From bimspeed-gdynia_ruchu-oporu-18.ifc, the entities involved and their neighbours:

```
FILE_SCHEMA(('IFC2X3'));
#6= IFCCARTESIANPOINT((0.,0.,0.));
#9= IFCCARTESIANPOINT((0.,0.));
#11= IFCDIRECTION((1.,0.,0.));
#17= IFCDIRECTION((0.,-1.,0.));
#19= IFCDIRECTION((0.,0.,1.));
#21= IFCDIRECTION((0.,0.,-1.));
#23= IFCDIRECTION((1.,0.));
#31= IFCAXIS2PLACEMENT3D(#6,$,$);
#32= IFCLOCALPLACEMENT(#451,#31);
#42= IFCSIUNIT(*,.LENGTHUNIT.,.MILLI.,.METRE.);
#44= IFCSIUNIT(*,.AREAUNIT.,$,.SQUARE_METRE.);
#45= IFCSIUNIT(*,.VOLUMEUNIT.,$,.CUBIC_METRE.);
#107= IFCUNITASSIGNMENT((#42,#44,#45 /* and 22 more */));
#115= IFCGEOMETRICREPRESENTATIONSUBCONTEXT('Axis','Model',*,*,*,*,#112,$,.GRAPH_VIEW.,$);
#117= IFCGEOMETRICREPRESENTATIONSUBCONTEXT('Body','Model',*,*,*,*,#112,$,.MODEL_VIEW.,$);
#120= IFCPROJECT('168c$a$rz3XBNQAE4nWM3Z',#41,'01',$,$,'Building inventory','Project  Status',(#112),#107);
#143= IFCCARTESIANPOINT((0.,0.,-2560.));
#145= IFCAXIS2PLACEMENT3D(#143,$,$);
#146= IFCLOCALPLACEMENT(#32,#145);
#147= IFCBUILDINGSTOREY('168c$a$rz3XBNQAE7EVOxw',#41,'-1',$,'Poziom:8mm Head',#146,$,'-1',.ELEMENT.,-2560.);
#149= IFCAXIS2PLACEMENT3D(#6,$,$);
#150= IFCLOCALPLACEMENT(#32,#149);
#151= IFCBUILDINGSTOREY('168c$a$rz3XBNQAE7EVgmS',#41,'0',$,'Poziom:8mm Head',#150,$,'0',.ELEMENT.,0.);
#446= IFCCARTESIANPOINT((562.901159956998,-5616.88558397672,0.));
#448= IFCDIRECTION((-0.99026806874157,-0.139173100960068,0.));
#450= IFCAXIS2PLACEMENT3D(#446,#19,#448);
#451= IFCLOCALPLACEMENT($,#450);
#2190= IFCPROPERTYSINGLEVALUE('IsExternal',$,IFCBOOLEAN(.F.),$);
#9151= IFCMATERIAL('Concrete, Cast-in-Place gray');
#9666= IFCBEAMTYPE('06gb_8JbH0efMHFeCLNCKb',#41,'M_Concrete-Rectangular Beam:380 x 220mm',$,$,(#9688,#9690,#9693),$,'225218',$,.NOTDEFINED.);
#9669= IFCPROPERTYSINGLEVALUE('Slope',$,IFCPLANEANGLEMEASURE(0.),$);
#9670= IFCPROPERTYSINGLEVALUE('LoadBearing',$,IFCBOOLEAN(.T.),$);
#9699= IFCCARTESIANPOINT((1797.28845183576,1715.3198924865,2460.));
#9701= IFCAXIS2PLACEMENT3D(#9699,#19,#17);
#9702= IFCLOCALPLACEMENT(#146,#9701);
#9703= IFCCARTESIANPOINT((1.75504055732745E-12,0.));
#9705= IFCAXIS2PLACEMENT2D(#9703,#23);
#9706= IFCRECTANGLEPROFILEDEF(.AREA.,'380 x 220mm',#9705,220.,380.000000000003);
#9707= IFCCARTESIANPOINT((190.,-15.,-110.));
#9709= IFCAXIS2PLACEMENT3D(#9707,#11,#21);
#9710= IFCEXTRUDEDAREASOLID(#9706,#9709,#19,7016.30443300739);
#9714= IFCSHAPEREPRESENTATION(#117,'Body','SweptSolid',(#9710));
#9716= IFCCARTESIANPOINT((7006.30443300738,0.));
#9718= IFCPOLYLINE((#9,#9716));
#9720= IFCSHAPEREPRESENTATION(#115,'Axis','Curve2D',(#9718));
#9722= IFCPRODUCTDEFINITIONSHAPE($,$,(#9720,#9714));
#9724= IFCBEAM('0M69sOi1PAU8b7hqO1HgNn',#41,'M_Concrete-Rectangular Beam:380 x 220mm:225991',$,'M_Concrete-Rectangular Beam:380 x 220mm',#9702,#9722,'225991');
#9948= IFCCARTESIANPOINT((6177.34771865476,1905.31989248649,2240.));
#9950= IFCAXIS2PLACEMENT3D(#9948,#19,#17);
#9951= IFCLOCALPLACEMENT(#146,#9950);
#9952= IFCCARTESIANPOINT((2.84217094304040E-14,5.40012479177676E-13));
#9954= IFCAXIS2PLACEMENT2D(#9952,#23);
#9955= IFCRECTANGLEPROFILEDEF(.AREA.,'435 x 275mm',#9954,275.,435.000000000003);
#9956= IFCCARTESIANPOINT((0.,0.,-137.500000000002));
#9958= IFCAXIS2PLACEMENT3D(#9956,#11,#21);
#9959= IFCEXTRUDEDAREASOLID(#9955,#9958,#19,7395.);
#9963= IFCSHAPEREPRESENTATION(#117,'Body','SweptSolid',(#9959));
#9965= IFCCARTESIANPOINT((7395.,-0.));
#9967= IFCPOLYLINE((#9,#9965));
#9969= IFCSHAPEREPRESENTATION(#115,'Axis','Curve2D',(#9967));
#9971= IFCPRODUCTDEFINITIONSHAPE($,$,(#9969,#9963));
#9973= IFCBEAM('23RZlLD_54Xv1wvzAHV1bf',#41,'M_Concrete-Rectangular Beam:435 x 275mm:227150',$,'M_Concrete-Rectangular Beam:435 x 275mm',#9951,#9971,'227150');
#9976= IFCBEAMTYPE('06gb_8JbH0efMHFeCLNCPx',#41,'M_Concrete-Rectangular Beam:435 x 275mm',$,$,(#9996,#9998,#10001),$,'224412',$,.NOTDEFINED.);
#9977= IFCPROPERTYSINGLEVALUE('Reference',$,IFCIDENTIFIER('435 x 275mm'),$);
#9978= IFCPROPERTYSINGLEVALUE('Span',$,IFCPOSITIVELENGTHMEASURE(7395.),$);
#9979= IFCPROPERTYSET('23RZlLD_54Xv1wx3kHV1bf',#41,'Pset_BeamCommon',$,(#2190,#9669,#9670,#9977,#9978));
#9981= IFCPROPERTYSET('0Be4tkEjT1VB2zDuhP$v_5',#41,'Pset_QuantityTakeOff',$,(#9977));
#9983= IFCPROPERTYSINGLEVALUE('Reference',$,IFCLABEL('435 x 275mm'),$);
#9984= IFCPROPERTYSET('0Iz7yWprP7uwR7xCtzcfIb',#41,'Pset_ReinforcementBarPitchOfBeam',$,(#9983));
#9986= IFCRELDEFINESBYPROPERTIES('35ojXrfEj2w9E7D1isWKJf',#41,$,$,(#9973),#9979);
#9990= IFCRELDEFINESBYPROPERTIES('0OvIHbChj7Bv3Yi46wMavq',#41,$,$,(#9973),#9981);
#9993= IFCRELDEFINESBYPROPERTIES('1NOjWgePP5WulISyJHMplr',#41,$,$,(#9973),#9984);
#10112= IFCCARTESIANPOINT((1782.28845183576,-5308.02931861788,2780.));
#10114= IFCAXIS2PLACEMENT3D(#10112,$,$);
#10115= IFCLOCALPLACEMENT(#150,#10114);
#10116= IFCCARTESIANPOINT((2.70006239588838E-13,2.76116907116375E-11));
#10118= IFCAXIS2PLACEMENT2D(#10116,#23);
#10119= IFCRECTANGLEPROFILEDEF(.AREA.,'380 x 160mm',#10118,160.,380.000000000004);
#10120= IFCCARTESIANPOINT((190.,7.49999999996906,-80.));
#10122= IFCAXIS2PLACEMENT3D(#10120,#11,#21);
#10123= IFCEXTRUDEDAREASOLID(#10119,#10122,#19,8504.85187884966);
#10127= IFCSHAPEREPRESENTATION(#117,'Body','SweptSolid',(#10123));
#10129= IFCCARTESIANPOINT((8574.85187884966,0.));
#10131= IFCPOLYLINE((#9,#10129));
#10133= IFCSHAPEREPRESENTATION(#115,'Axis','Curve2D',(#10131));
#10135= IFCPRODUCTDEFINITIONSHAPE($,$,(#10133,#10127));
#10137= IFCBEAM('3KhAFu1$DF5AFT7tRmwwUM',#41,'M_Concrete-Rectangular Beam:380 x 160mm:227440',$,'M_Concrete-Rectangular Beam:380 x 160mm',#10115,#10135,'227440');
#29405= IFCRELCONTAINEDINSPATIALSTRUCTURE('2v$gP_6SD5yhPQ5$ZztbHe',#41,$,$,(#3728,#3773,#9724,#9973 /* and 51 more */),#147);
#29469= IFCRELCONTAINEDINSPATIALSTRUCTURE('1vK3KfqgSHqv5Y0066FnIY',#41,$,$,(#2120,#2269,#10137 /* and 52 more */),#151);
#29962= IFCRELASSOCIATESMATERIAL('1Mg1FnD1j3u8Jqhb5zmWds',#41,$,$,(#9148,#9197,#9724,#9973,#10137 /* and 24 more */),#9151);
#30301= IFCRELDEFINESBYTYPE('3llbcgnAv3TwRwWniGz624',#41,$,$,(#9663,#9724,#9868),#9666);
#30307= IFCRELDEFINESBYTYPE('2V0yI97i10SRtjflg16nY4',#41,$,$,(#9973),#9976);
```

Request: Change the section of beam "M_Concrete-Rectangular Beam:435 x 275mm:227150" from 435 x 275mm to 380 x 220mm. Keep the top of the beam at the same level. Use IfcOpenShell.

```python
import ifcopenshell
import ifcopenshell.api.pset
import ifcopenshell.api.type
import ifcopenshell.util.element
import ifcopenshell.util.representation

model = ifcopenshell.open("bimspeed-gdynia_ruchu-oporu-18.ifc")

member = model.by_guid("23RZlLD_54Xv1wvzAHV1bf")
source = next(p for p in model.by_type("IfcRectangleProfileDef") if p.ProfileName == "380 x 220mm")

body = ifcopenshell.util.representation.get_representation(member, "Model", "Body")
solid = body.Items[0]
old_profile = solid.SweptArea

# Copy the section's sizes but keep this member's own profile position.
profile = ifcopenshell.util.element.copy(model, source)
# Profiles are centred, so shift by half the change in depth to hold the top.
shift = (old_profile.XDim - profile.XDim) / 2
x, y = old_profile.Position.Location.Coordinates
up = (-1.0, 0.0)  # upwards, in the solid's own plane
location = model.createIfcCartesianPoint((x + up[0] * shift, y + up[1] * shift))
profile.Position = model.createIfcAxis2Placement2D(location, old_profile.Position.RefDirection)
solid.SweptArea = profile
if not model.get_total_inverses(old_profile):
    ifcopenshell.util.element.remove_deep2(model, old_profile)

new_type = model.by_id(9666)
ifcopenshell.api.type.assign_type(
    model, related_objects=[member], relating_type=new_type, should_map_representations=False
)
member.Name = member.Name.replace("435 x 275mm", "380 x 220mm")
member.ObjectType = "M_Concrete-Rectangular Beam:380 x 220mm"
pset = model.by_id(ifcopenshell.util.element.get_pset(member, "Pset_BeamCommon", should_inherit=False)["id"])
ifcopenshell.api.pset.edit_pset(model, pset=pset, properties={"Reference": "380 x 220mm"})
pset = model.by_id(ifcopenshell.util.element.get_pset(member, "Pset_QuantityTakeOff", should_inherit=False)["id"])
ifcopenshell.api.pset.edit_pset(model, pset=pset, properties={"Reference": "380 x 220mm"})
pset = model.by_id(ifcopenshell.util.element.get_pset(member, "Pset_ReinforcementBarPitchOfBeam", should_inherit=False)["id"])
ifcopenshell.api.pset.edit_pset(model, pset=pset, properties={"Reference": "380 x 220mm"})

print(solid.SweptArea)

model.write("bimspeed-gdynia_ruchu-oporu-18_v2.ifc")
```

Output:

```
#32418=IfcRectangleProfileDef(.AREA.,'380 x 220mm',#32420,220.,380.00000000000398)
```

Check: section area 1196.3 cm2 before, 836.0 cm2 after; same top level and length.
